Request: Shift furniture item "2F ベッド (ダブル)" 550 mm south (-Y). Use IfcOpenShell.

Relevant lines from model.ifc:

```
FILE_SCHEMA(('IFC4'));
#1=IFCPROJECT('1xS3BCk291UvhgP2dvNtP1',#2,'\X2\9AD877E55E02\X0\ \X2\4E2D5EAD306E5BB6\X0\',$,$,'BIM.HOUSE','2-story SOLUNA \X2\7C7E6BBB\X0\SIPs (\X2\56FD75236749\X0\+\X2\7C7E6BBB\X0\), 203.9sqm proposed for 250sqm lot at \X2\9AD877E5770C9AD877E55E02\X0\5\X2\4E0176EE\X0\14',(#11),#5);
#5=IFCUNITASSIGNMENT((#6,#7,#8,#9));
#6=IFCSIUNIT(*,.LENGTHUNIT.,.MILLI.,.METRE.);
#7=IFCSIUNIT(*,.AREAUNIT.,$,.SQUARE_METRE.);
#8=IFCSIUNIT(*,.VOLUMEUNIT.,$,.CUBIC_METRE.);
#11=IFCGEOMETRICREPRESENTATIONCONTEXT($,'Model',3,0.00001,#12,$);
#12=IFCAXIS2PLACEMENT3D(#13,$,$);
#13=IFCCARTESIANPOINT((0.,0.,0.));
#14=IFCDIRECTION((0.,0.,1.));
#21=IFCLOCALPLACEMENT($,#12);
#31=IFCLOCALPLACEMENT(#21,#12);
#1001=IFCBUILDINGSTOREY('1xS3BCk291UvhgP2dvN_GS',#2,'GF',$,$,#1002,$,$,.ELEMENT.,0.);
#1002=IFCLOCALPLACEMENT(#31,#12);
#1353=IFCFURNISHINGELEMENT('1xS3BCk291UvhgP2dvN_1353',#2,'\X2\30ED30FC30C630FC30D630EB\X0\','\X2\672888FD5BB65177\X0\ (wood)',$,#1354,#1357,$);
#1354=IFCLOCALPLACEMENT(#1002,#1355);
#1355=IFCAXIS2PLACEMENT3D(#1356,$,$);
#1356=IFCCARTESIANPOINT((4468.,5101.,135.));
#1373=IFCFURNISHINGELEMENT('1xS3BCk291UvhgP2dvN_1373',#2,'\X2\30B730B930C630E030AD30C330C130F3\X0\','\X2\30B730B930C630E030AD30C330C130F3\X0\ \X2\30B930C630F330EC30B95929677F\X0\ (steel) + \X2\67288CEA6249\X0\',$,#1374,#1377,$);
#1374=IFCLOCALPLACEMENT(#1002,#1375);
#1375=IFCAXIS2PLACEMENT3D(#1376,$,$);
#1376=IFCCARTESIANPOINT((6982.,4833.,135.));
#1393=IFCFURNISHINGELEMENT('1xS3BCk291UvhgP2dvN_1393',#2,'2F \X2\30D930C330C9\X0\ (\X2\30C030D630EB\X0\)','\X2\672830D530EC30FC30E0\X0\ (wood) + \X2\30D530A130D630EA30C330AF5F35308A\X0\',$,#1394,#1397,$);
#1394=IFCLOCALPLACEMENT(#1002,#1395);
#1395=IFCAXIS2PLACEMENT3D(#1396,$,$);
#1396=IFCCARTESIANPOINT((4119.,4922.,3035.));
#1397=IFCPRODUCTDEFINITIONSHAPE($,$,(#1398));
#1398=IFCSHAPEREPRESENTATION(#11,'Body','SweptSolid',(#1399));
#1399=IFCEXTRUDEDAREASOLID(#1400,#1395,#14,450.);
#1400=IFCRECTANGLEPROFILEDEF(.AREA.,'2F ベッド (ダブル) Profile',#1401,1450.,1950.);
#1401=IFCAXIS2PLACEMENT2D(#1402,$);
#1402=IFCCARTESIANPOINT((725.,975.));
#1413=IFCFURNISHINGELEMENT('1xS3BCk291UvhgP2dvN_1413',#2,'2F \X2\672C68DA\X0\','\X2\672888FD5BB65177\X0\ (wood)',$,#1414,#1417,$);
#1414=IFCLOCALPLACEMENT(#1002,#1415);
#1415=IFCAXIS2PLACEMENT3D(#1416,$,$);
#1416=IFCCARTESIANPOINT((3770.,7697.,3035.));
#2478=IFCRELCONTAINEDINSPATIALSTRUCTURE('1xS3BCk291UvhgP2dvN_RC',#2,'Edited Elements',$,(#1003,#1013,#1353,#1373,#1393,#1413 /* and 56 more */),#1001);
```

```python
import ifcopenshell
import ifcopenshell.api.geometry
import ifcopenshell.util.placement

model = ifcopenshell.open("model.ifc")

item = model.by_guid("1xS3BCk291UvhgP2dvN_1393")
matrix = ifcopenshell.util.placement.get_local_placement(item.ObjectPlacement)
matrix[1, 3] -= 550.0
ifcopenshell.api.geometry.edit_object_placement(model, product=item, matrix=matrix, is_si=False)

print(ifcopenshell.util.placement.get_local_placement(item.ObjectPlacement).round(3) + 0.0)

model.write("model-out.ifc")
```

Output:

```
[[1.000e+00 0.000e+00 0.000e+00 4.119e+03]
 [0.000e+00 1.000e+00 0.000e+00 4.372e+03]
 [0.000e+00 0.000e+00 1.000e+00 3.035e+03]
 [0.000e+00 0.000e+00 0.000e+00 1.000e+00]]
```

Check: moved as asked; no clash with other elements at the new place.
